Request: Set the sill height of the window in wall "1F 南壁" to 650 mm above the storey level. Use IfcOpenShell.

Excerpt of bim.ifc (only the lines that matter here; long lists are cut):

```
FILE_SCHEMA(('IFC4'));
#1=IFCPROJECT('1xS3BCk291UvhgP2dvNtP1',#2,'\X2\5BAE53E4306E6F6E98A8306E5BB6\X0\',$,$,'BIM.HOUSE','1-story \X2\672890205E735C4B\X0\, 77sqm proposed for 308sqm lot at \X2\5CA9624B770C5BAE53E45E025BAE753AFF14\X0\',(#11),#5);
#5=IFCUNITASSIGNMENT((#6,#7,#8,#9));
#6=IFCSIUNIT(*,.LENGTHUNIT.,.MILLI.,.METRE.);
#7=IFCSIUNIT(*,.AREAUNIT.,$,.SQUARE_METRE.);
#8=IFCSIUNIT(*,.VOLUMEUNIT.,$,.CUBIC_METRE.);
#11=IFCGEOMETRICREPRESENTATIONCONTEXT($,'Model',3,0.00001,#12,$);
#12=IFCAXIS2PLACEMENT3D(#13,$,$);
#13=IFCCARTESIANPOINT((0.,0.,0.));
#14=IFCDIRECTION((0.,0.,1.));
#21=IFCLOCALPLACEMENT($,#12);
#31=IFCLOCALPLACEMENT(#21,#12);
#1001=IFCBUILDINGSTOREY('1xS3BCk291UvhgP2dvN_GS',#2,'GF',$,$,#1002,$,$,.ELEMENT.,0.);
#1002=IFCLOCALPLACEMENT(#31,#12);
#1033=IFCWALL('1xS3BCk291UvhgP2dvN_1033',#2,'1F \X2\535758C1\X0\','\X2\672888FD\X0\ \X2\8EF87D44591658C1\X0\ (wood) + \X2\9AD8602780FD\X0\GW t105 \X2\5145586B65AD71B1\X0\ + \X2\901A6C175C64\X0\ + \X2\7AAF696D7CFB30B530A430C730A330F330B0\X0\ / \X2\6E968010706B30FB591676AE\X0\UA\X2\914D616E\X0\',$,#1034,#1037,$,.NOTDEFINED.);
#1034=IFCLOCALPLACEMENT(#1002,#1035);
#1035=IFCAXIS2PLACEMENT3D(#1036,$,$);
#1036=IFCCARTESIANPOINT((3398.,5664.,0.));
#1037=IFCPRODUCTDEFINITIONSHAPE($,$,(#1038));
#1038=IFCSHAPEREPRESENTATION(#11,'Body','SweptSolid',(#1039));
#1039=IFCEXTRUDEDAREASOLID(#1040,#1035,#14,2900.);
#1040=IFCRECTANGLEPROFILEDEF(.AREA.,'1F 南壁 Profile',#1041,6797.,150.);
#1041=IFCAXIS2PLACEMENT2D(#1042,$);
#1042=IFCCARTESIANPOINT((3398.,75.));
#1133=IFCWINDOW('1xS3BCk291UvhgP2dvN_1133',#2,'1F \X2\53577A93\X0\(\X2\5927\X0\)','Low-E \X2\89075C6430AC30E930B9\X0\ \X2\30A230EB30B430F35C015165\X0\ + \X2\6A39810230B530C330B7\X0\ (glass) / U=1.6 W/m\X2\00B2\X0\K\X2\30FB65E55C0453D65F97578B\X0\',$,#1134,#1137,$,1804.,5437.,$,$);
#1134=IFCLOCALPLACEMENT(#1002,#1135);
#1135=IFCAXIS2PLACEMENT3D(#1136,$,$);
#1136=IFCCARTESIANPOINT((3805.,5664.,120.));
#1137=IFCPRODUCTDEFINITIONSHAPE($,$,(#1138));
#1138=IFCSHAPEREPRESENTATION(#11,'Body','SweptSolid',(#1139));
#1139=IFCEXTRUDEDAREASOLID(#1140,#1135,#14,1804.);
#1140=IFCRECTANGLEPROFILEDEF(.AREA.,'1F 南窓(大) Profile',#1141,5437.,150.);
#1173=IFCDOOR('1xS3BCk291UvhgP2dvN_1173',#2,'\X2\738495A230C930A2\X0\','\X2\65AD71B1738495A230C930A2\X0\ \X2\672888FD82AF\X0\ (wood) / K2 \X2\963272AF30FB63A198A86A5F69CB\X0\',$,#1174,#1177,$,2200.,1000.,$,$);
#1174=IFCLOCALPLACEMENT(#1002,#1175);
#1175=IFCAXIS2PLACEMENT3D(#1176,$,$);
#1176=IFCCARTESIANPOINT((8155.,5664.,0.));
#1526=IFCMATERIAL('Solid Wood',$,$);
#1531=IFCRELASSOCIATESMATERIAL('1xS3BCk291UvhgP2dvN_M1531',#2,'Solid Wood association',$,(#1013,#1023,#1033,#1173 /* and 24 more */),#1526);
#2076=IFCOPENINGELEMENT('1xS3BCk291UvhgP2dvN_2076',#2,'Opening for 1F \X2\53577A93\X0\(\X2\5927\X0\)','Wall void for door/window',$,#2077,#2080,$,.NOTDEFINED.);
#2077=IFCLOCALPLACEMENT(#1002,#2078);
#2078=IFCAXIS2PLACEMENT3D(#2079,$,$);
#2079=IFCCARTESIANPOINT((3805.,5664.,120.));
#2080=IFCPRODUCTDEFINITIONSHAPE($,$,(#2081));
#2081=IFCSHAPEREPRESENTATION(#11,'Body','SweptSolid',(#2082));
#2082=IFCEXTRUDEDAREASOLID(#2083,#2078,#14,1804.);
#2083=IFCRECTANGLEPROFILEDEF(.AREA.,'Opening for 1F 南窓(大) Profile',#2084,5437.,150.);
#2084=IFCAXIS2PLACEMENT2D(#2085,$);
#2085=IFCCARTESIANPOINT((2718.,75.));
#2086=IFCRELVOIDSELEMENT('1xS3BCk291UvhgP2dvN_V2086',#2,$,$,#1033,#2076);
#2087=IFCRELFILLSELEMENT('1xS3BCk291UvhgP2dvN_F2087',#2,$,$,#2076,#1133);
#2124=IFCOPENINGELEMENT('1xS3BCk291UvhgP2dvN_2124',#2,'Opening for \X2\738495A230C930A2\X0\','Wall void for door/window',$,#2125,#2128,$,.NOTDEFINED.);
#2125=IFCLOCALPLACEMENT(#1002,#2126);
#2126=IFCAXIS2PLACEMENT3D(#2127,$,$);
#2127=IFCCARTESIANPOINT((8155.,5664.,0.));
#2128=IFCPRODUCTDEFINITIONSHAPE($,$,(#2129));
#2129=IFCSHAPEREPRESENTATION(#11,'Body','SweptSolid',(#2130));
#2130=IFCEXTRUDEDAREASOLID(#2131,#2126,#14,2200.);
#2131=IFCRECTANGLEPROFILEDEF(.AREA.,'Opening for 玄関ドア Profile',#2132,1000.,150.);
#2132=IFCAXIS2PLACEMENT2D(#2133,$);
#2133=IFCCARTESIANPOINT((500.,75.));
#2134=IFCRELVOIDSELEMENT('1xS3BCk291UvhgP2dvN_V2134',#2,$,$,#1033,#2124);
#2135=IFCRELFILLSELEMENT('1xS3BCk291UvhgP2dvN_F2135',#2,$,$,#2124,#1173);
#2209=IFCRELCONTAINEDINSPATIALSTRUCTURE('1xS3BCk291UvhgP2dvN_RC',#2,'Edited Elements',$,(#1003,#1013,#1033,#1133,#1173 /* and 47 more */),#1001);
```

```python
import numpy as np
import ifcopenshell
import ifcopenshell.api.geometry
import ifcopenshell.geom
import ifcopenshell.util.element
import ifcopenshell.util.placement
import ifcopenshell.util.shape
import ifcopenshell.util.unit

model = ifcopenshell.open("bim.ifc")
unit_scale = ifcopenshell.util.unit.calculate_unit_scale(model)

window = model.by_guid("1xS3BCk291UvhgP2dvN_1133")
opening = window.FillsVoids[0].RelatingOpeningElement
storey = ifcopenshell.util.element.get_container(window, ifc_class="IfcBuildingStorey")
level = ifcopenshell.util.placement.get_local_placement(storey.ObjectPlacement)[2, 3]

# The opening's origin need not be at the sill, so measure its lowest point.
shape = ifcopenshell.geom.create_shape(ifcopenshell.geom.settings(), opening)
bottom = ifcopenshell.util.shape.get_shape_bottom_elevation(shape, shape.geometry) / unit_scale
dz = level + 650.0 - bottom

shift = np.array([0.0, 0.0, dz])
# The window is not placed relative to its opening, so move both.
for product in (opening, window):
    matrix = ifcopenshell.util.placement.get_local_placement(product.ObjectPlacement)
    matrix[:3, 3] += shift
    ifcopenshell.api.geometry.edit_object_placement(model, product=product, matrix=matrix, is_si=False)

print(f"moved by {dz * unit_scale:+.3f} m")

model.write("bim-out.ifc")
```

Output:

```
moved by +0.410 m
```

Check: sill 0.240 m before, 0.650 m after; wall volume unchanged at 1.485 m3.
